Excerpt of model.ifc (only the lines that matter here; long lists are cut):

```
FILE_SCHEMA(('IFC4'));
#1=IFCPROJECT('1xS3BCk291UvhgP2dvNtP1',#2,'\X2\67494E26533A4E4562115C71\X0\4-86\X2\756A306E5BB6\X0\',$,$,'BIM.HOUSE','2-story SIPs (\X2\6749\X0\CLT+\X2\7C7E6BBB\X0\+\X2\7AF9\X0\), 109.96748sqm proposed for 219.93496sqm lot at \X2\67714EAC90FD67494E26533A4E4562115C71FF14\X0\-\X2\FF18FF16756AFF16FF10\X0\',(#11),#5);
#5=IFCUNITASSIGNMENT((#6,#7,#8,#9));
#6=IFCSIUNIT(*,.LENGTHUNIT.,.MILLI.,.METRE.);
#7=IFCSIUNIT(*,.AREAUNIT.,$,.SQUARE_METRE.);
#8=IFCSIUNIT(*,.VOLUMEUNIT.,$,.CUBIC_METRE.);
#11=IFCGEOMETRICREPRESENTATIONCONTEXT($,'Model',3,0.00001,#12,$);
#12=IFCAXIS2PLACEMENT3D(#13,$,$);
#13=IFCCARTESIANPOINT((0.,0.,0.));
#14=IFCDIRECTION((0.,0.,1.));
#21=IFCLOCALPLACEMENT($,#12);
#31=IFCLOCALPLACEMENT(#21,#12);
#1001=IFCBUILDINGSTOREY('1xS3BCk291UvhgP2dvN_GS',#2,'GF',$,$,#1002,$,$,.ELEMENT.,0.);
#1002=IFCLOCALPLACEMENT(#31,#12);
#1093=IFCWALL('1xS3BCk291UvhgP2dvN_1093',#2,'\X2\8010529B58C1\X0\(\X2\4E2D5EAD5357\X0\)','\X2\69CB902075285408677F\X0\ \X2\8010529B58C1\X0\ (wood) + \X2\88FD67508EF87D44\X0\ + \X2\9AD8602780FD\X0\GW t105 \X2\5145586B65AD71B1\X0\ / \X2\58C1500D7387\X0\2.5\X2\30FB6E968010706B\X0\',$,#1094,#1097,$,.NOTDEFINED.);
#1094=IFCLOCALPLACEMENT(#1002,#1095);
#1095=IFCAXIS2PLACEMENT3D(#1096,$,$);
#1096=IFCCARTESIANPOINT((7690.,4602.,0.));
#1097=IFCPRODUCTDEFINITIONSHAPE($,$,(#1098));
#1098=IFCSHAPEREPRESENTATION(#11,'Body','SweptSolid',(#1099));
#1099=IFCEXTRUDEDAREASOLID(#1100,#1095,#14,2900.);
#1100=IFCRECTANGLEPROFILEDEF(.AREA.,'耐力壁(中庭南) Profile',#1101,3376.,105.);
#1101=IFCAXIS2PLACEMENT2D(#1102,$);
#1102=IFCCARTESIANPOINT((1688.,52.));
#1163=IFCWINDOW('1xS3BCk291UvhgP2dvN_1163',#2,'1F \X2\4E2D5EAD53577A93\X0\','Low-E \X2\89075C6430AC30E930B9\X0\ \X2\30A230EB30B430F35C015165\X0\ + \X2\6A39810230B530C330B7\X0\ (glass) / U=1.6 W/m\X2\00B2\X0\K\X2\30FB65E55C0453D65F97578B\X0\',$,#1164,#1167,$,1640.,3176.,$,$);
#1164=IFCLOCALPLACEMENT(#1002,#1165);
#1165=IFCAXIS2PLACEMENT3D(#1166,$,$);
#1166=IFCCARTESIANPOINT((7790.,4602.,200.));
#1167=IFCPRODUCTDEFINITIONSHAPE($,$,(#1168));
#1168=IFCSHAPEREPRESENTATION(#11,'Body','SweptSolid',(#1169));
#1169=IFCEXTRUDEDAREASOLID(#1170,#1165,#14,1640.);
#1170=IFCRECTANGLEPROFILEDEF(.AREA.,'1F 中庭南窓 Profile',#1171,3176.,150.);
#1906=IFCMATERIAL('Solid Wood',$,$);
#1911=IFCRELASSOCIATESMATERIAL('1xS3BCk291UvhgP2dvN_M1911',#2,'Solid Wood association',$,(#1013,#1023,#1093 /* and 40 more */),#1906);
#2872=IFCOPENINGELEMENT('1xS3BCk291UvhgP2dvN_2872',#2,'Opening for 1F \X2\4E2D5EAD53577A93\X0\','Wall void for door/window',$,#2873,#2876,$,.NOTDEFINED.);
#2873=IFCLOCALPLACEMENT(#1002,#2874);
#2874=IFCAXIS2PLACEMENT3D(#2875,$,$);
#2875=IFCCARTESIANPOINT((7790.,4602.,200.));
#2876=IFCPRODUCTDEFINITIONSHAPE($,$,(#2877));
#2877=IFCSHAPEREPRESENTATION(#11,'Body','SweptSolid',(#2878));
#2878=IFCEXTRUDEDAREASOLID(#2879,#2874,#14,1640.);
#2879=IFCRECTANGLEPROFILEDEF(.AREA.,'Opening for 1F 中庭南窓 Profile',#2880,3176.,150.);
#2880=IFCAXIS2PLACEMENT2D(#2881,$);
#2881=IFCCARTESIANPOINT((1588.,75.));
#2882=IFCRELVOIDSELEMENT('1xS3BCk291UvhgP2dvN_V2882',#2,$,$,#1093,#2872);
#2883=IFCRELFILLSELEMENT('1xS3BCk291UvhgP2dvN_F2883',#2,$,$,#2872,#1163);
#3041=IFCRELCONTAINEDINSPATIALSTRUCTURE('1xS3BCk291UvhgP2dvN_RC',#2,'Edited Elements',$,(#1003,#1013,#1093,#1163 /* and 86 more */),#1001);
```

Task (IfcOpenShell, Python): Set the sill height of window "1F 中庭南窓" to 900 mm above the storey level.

```python
import numpy as np
import ifcopenshell
import ifcopenshell.api.geometry
import ifcopenshell.geom
import ifcopenshell.util.element
import ifcopenshell.util.placement
import ifcopenshell.util.shape
import ifcopenshell.util.unit

model = ifcopenshell.open("model.ifc")
unit_scale = ifcopenshell.util.unit.calculate_unit_scale(model)

window = model.by_guid("1xS3BCk291UvhgP2dvN_1163")
opening = window.FillsVoids[0].RelatingOpeningElement
storey = ifcopenshell.util.element.get_container(window, ifc_class="IfcBuildingStorey")
level = ifcopenshell.util.placement.get_local_placement(storey.ObjectPlacement)[2, 3]

# The opening's origin need not be at the sill, so measure its lowest point.
shape = ifcopenshell.geom.create_shape(ifcopenshell.geom.settings(), opening)
bottom = ifcopenshell.util.shape.get_shape_bottom_elevation(shape, shape.geometry) / unit_scale
dz = level + 0.9 / unit_scale - bottom

shift = np.array([0.0, 0.0, dz])
# The window is not placed relative to its opening, so move both.
for product in (opening, window):
    matrix = ifcopenshell.util.placement.get_local_placement(product.ObjectPlacement)
    matrix[:3, 3] += shift
    ifcopenshell.api.geometry.edit_object_placement(model, product=product, matrix=matrix, is_si=False)

print(f"moved by {dz * unit_scale:+.3f} m")

model.write("model_rev.ifc")
```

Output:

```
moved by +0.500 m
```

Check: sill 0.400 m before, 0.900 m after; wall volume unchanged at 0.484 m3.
